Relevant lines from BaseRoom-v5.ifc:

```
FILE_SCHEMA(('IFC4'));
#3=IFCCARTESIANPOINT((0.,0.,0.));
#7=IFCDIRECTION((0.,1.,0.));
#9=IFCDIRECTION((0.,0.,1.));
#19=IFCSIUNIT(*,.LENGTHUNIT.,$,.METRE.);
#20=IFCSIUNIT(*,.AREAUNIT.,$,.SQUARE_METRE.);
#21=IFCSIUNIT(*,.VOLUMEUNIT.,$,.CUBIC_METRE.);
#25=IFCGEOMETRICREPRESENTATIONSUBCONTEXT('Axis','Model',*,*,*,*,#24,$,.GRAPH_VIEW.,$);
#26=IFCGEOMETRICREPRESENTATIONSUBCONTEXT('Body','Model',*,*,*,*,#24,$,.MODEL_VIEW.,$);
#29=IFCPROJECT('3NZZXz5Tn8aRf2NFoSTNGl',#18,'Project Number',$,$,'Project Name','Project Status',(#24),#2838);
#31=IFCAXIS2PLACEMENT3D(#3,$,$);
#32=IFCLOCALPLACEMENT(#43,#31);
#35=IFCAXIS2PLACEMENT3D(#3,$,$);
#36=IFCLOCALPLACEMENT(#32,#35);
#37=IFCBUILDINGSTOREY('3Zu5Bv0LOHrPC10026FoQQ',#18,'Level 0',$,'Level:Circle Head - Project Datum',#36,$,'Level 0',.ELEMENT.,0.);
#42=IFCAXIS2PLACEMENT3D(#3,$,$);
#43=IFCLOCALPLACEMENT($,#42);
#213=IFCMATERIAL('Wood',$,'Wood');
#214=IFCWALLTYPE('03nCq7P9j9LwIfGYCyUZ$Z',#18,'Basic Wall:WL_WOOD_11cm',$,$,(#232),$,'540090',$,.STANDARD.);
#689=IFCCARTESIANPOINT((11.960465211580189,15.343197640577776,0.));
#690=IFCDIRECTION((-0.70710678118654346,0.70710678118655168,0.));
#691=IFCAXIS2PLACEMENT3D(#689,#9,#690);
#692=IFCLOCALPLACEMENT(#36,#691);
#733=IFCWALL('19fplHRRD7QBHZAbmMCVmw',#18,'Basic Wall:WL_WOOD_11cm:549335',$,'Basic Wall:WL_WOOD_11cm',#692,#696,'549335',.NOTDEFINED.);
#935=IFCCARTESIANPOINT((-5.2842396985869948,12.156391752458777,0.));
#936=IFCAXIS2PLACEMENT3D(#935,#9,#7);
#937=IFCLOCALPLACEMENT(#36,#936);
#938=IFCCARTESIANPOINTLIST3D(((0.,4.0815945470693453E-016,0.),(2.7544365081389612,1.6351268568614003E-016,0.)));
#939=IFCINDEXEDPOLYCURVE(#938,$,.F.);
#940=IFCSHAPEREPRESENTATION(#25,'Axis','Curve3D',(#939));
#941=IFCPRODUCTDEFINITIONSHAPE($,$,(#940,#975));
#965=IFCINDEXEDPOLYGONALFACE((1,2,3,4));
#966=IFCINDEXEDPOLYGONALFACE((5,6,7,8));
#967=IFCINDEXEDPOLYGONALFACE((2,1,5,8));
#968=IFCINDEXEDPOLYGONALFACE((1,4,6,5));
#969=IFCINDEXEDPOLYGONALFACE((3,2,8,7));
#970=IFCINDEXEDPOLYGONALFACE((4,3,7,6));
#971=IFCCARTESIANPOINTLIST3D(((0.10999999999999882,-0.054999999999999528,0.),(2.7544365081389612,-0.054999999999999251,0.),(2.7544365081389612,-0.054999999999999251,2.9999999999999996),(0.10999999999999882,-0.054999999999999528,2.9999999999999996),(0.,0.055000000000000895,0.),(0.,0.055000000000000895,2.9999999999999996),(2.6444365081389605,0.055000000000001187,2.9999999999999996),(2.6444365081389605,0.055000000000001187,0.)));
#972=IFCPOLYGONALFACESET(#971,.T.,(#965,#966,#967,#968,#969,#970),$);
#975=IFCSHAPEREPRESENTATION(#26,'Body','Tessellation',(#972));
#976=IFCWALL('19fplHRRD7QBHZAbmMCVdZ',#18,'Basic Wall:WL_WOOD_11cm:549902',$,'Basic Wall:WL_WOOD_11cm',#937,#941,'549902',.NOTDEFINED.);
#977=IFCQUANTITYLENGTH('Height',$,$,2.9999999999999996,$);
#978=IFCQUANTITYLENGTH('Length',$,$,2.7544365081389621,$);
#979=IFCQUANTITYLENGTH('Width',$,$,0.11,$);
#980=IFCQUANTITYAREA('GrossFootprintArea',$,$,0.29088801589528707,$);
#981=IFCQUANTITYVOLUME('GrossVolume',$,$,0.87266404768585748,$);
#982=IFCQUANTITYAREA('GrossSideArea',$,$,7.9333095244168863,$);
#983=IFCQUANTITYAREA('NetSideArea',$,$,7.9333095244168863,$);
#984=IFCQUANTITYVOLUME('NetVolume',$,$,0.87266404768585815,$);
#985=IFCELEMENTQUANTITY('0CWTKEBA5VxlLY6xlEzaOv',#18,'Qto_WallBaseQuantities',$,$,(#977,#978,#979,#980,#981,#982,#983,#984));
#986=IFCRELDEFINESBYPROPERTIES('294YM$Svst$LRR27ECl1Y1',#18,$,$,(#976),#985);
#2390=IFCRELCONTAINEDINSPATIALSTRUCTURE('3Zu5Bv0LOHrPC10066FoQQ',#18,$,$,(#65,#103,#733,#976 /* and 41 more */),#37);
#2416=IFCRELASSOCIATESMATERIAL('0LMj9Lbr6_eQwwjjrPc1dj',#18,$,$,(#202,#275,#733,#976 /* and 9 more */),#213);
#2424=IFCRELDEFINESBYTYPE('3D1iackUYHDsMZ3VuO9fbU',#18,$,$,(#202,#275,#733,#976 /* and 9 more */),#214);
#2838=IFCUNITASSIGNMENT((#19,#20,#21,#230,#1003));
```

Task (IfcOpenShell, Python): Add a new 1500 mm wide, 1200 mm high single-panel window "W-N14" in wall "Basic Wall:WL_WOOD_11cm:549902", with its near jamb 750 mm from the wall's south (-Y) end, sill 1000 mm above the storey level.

```python
import numpy as np
import ifcopenshell
import ifcopenshell.api.feature
import ifcopenshell.api.geometry
import ifcopenshell.api.pset
import ifcopenshell.api.root
import ifcopenshell.api.spatial
import ifcopenshell.geom
import ifcopenshell.util.element
import ifcopenshell.util.placement
import ifcopenshell.util.representation
import ifcopenshell.util.shape
import ifcopenshell.util.unit

model = ifcopenshell.open("BaseRoom-v5.ifc")
unit_scale = ifcopenshell.util.unit.calculate_unit_scale(model)
area_scale = ifcopenshell.util.unit.calculate_unit_scale(model, "AREAUNIT")
volume_scale = ifcopenshell.util.unit.calculate_unit_scale(model, "VOLUMEUNIT")
settings = ifcopenshell.geom.settings()


def volume(element):
    """Net volume in cubic metres, openings subtracted."""
    shape = ifcopenshell.geom.create_shape(settings, element)
    return ifcopenshell.util.shape.get_volume(shape.geometry)


wall = model.by_guid("19fplHRRD7QBHZAbmMCVdZ")
storey = ifcopenshell.util.element.get_container(wall, ifc_class="IfcBuildingStorey")
context = ifcopenshell.util.representation.get_context(model, "Model", "Body", "MODEL_VIEW")
before = volume(wall)

width, height, from_end, sill = 1.5, 1.2, 0.75, 1  # metres

# The wall runs along its own X axis, and the end named is its -X end.
wall_shape = ifcopenshell.geom.create_shape(settings, wall)
x, y, z = ifcopenshell.util.shape.get_vertices(wall_shape.geometry).T
start = x.min() + from_end
face, thickness = float(y.min()), float(y.max() - y.min())
wall_matrix = ifcopenshell.util.placement.get_local_placement(wall.ObjectPlacement)
level = ifcopenshell.util.placement.get_local_placement(storey.ObjectPlacement)[2, 3]


def in_wall(x, y):
    """Placement at x, y metres in the wall's axes, at sill height."""
    matrix = wall_matrix.copy()
    matrix[:, 3] = wall_matrix @ np.array([x / unit_scale, y / unit_scale, 0.0, 1.0])
    matrix[2, 3] = level + sill / unit_scale
    return matrix


# Opening: a box that overshoots both wall faces by 50 mm.
opening = ifcopenshell.api.root.create_entity(model, ifc_class="IfcOpeningElement", predefined_type="OPENING")
box = ifcopenshell.api.geometry.add_wall_representation(
    model, context=context, length=width, height=height, thickness=thickness + 0.1
)
ifcopenshell.api.geometry.assign_representation(model, product=opening, representation=box)
ifcopenshell.api.geometry.edit_object_placement(model, product=opening, matrix=in_wall(start, face - 0.05), is_si=False)
ifcopenshell.api.feature.add_feature(model, feature=opening, element=wall)

window = ifcopenshell.api.root.create_entity(model, ifc_class="IfcWindow", name="W-N14", predefined_type="WINDOW")
window.OverallWidth, window.OverallHeight = width / unit_scale, height / unit_scale
window.PartitioningType = "SINGLE_PANEL"
body = ifcopenshell.api.geometry.add_window_representation(
    model,
    context=context,
    overall_width=window.OverallWidth,
    overall_height=window.OverallHeight,
    partition_type="SINGLE_PANEL",
)
ifcopenshell.api.geometry.assign_representation(model, product=window, representation=body)
ifcopenshell.api.spatial.assign_container(model, products=[window], relating_structure=storey)
ifcopenshell.api.feature.add_filling(model, opening=opening, element=window)

# Centre the window in the wall's thickness.
ifcopenshell.api.geometry.edit_object_placement(model, product=window, matrix=in_wall(start, face), is_si=False)
window_shape = ifcopenshell.geom.create_shape(settings, window)
depth = ifcopenshell.util.shape.get_vertices(window_shape.geometry)[:, 1]
offset = face + thickness / 2 - (depth.min() + depth.max()) / 2
ifcopenshell.api.geometry.edit_object_placement(model, product=window, matrix=in_wall(start, offset), is_si=False)

after = volume(wall)

# Update the wall's stored quantities.
qto = model.by_id(ifcopenshell.util.element.get_pset(wall, "Qto_WallBaseQuantities", should_inherit=False)["id"])
ifcopenshell.api.pset.edit_qto(model, qto=qto, properties={
    "NetSideArea": after / thickness / area_scale,
    "NetVolume": after / volume_scale,
})

print(f"wall volume {before:.3f} -> {after:.3f} m3")

model.write("BaseRoom-v5_updated.ifc")
```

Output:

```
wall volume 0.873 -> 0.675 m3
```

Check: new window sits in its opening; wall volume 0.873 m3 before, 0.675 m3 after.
